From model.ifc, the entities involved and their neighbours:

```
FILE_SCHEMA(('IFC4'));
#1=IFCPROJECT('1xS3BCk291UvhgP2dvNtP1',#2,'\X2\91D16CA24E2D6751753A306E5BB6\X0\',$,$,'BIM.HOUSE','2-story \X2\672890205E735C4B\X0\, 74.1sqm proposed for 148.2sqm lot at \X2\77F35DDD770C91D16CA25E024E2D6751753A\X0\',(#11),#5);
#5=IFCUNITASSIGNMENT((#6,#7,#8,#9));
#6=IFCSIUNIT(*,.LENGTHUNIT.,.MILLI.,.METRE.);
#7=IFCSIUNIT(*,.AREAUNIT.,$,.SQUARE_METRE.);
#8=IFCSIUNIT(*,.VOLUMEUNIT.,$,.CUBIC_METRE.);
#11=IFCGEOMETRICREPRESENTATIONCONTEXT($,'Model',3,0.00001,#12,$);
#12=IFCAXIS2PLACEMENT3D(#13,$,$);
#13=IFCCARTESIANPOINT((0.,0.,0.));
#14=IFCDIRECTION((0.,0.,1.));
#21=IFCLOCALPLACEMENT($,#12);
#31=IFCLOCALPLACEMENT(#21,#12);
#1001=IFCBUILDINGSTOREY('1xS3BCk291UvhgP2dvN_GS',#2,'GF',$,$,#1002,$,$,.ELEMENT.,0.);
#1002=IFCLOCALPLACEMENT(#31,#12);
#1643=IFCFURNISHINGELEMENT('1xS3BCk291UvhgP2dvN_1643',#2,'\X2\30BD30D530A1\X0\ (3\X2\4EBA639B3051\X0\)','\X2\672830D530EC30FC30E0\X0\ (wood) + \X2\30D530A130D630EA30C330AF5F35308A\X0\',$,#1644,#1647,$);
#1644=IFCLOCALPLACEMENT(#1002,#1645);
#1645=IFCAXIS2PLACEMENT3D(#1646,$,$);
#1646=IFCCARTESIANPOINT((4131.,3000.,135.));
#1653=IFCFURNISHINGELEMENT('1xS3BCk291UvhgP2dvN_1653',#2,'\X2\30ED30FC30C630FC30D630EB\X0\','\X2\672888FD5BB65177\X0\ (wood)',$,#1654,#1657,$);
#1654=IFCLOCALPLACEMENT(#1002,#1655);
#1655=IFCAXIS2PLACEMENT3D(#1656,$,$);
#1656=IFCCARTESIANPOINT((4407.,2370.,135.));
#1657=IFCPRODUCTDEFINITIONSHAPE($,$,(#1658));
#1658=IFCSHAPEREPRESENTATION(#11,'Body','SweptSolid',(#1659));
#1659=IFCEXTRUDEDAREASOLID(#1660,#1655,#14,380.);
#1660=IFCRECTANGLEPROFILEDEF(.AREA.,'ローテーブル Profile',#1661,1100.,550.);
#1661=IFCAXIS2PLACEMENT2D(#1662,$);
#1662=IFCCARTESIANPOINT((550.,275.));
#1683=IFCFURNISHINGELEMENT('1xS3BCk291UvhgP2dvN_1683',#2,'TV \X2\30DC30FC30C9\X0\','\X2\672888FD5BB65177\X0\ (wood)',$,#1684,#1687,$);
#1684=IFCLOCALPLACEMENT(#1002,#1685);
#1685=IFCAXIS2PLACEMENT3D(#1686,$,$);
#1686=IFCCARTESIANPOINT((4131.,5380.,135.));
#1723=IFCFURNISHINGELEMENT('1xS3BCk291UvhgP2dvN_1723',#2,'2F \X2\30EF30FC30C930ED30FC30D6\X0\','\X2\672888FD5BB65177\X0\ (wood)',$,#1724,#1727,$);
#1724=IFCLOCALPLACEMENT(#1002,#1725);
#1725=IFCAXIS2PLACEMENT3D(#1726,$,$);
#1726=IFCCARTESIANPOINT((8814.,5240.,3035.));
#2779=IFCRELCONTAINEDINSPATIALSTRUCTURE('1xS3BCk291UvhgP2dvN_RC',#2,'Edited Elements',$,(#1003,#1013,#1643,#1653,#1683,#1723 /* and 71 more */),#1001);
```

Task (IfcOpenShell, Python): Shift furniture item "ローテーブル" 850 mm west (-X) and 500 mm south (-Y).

```python
import ifcopenshell
import ifcopenshell.api.geometry
import ifcopenshell.util.placement
import ifcopenshell.util.unit

model = ifcopenshell.open("model.ifc")
unit_scale = ifcopenshell.util.unit.calculate_unit_scale(model)

item = model.by_guid("1xS3BCk291UvhgP2dvN_1653")
matrix = ifcopenshell.util.placement.get_local_placement(item.ObjectPlacement)
matrix[0, 3] -= 0.85 / unit_scale
matrix[1, 3] -= 0.5 / unit_scale
ifcopenshell.api.geometry.edit_object_placement(model, product=item, matrix=matrix, is_si=False)

print(ifcopenshell.util.placement.get_local_placement(item.ObjectPlacement).round(3) + 0.0)

model.write("model_v2.ifc")
```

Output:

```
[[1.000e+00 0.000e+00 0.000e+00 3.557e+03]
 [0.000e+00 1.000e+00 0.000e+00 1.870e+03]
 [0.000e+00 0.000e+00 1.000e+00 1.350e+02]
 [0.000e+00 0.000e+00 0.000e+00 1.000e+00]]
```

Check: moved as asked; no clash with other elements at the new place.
